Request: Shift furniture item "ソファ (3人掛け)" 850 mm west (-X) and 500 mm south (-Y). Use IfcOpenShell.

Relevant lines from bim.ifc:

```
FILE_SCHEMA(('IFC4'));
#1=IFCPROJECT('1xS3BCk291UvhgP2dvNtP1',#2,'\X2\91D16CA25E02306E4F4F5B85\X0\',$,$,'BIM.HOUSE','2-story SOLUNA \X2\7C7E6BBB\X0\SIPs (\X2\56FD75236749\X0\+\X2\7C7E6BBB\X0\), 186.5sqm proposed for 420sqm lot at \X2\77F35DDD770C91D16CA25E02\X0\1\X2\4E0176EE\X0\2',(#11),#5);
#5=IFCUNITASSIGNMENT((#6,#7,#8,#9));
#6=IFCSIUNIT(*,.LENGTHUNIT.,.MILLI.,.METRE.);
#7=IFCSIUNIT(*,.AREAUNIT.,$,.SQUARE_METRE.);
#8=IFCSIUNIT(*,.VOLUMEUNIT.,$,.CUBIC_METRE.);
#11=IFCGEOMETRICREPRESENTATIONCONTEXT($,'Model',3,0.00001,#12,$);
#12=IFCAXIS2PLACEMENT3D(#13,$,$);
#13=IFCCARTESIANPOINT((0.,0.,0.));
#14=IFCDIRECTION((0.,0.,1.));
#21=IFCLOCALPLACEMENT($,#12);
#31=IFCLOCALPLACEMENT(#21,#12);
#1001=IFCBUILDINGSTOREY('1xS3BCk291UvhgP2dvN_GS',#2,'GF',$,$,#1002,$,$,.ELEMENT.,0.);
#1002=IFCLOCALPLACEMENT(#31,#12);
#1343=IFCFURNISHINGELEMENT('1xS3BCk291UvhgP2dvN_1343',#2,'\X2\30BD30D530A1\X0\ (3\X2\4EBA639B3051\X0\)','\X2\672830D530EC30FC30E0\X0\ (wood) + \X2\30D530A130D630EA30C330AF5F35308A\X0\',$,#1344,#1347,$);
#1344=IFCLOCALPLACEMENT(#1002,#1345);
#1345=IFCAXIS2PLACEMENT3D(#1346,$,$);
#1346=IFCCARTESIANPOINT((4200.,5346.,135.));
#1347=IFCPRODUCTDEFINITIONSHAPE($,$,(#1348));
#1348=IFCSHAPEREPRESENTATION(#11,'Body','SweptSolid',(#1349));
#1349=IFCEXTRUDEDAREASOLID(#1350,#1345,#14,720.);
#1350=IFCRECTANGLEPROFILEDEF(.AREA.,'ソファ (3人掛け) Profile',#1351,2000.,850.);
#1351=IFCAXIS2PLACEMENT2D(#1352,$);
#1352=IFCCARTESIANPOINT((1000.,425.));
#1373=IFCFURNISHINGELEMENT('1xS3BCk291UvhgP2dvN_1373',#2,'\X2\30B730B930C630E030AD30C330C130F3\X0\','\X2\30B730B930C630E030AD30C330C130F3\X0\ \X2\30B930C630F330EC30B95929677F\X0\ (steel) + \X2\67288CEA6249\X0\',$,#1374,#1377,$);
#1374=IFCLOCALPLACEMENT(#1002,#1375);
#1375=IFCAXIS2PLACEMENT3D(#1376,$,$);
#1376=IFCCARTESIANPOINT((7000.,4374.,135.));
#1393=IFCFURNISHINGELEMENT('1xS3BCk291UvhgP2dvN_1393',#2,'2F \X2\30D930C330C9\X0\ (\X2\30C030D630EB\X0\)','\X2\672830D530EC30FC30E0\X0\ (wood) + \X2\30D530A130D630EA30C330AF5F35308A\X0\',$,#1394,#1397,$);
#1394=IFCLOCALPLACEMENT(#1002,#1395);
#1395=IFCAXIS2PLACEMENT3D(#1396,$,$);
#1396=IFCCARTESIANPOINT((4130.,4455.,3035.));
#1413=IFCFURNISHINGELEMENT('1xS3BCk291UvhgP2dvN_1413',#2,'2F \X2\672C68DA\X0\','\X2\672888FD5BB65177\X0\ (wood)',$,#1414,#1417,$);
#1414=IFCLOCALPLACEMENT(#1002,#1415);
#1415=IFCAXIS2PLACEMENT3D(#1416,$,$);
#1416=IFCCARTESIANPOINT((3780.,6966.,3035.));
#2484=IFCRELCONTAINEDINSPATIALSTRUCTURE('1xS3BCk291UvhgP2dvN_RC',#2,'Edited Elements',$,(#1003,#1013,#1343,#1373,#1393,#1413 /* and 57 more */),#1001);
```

```python
import ifcopenshell
import ifcopenshell.api.geometry
import ifcopenshell.util.placement
import ifcopenshell.util.unit

model = ifcopenshell.open("bim.ifc")
unit_scale = ifcopenshell.util.unit.calculate_unit_scale(model)

item = model.by_guid("1xS3BCk291UvhgP2dvN_1343")
matrix = ifcopenshell.util.placement.get_local_placement(item.ObjectPlacement)
matrix[0, 3] -= 0.85 / unit_scale
matrix[1, 3] -= 0.5 / unit_scale
ifcopenshell.api.geometry.edit_object_placement(model, product=item, matrix=matrix, is_si=False)

print(ifcopenshell.util.placement.get_local_placement(item.ObjectPlacement).round(3) + 0.0)

model.write("bim_edited.ifc")
```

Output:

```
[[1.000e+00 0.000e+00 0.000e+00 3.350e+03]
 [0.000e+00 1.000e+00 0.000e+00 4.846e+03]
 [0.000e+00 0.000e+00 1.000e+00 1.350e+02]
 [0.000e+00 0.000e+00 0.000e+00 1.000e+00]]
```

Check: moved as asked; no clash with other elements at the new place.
